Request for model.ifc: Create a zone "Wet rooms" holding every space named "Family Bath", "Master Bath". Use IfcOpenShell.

First a look at what the model holds.

```python
import ifcopenshell

model = ifcopenshell.open("model.ifc")
print(model.schema)
seen = {}
for space in model.by_type("IfcSpace"):
    seen[space.LongName] = seen.get(space.LongName, 0) + 1
for name, count in sorted(seen.items(), key=str):
    print(count, "x", name)
print("zones:", [z.Name for z in model.by_type("IfcZone")][:20])
```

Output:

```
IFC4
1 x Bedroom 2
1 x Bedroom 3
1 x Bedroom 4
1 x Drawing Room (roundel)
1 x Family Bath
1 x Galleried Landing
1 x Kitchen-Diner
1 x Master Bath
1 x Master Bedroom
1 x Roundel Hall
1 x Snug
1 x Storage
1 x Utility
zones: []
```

```python
import ifcopenshell
import ifcopenshell.api.group
import ifcopenshell.api.root

model = ifcopenshell.open("model.ifc")

names = {"Family Bath", "Master Bath"}
spaces = [s for s in model.by_type("IfcSpace") if s.LongName in names]

zone = ifcopenshell.api.root.create_entity(model, ifc_class="IfcZone", name="Wet rooms")
ifcopenshell.api.group.assign_group(model, products=spaces, group=zone)
print(len(spaces), "spaces in", zone.Name)

model.write("model_rev.ifc")
```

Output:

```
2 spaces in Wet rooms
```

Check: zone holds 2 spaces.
